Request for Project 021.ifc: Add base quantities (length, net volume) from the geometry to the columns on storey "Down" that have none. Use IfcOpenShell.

First a look at what the model holds.

```python
import ifcopenshell
import ifcopenshell.util.element
import ifcopenshell.util.unit

model = ifcopenshell.open("Project 021.ifc")
print(model.schema)
for unit_type in ("LENGTHUNIT", "AREAUNIT", "VOLUMEUNIT"):
    print(unit_type, ifcopenshell.util.unit.calculate_unit_scale(model, unit_type))
storey = next(s for s in model.by_type("IfcBuildingStorey") if s.Name == "Down")
columns = [e for e in ifcopenshell.util.element.get_decomposition(storey) if e.is_a("IfcColumn")]
for e in sorted(columns, key=lambda e: e.id()):
    print(e.id(), e.is_a(), e.Name, list(ifcopenshell.util.element.get_psets(e, qtos_only=True)), sep=" | ")
```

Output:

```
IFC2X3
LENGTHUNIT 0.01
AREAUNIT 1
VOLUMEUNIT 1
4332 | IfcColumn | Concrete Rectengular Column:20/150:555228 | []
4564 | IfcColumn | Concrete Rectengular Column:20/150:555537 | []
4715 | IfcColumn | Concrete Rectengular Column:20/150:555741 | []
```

```python
import ifcopenshell
import ifcopenshell.api.pset
import ifcopenshell.geom
import ifcopenshell.util.element
import ifcopenshell.util.shape
import ifcopenshell.util.unit

model = ifcopenshell.open("Project 021.ifc")
unit_scale = ifcopenshell.util.unit.calculate_unit_scale(model)
volume_scale = ifcopenshell.util.unit.calculate_unit_scale(model, "VOLUMEUNIT")
settings = ifcopenshell.geom.settings()

storey = next(s for s in model.by_type("IfcBuildingStorey") if s.Name == "Down")
columns = [e for e in ifcopenshell.util.element.get_decomposition(storey) if e.is_a("IfcColumn")]

for e in sorted(columns, key=lambda e: e.id()):
    if ifcopenshell.util.element.get_psets(e, qtos_only=True, should_inherit=False):
        continue
    # Geometry comes back in metres, in the element's own axes.
    shape = ifcopenshell.geom.create_shape(settings, e)
    values = {
        "Length": ifcopenshell.util.shape.get_z(shape.geometry) / unit_scale,
        "NetVolume": ifcopenshell.util.shape.get_volume(shape.geometry) / volume_scale,
    }
    qto = ifcopenshell.api.pset.add_qto(model, product=e, name="BaseQuantities")
    ifcopenshell.api.pset.edit_qto(model, qto=qto, properties=values)
    print(e.id(), {k: round(v, 3) for k, v in values.items()})

model.write("Project 021_updated.ifc")
```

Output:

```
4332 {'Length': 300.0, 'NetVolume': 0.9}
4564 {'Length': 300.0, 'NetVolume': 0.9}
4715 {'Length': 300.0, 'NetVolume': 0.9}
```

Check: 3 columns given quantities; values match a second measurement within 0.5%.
